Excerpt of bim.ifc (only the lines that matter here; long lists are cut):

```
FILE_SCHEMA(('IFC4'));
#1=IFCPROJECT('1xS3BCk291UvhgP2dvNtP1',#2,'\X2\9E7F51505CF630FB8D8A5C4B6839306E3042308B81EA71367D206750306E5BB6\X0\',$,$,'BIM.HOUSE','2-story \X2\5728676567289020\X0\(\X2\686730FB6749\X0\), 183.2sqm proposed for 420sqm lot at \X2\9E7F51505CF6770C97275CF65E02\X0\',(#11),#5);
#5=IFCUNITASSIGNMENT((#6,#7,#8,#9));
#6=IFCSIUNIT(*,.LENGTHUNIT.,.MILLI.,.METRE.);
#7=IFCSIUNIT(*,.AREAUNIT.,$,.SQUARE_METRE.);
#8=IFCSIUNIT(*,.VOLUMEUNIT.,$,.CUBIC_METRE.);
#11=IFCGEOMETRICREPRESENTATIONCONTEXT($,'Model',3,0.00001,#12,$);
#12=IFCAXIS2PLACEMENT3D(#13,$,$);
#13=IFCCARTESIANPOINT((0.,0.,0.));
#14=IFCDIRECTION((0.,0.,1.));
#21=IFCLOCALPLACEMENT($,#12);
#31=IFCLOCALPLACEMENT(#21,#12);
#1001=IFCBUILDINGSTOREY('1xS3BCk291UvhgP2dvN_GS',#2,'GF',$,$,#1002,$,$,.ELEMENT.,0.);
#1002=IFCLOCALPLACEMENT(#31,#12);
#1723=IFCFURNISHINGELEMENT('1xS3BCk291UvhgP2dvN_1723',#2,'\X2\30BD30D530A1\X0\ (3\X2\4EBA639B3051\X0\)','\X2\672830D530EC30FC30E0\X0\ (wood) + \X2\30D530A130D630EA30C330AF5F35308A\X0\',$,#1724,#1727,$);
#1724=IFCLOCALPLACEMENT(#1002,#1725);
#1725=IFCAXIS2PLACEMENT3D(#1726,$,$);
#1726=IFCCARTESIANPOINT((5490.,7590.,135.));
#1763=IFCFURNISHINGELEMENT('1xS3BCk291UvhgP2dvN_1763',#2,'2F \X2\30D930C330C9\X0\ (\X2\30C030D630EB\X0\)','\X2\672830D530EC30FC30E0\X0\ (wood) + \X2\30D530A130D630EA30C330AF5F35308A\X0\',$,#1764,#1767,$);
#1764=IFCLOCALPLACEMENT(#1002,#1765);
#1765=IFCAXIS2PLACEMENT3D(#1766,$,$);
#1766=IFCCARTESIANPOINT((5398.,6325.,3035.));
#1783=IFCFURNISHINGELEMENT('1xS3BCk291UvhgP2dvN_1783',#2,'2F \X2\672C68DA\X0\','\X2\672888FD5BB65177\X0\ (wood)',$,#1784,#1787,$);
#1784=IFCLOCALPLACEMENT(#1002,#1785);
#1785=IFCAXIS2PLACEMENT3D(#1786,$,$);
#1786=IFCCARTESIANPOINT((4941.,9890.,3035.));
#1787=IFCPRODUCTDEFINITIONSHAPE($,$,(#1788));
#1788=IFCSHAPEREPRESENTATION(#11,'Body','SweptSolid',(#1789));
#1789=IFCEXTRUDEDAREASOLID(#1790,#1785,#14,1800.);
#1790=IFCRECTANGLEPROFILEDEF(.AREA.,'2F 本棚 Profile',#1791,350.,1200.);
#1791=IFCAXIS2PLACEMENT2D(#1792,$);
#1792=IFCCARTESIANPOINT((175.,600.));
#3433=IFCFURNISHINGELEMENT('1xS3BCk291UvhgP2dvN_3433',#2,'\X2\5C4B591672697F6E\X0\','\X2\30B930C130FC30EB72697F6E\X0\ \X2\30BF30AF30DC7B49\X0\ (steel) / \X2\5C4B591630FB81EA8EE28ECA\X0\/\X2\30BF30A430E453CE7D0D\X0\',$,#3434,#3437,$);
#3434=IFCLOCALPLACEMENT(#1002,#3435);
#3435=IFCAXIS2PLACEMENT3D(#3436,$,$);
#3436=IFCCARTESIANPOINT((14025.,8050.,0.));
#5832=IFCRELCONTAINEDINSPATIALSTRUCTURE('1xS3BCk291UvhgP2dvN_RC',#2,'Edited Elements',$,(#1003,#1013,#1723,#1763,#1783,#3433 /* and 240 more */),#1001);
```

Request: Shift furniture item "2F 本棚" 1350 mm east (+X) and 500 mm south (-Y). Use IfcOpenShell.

```python
import ifcopenshell
import ifcopenshell.api.geometry
import ifcopenshell.util.placement
import ifcopenshell.util.unit

model = ifcopenshell.open("bim.ifc")
unit_scale = ifcopenshell.util.unit.calculate_unit_scale(model)

item = model.by_guid("1xS3BCk291UvhgP2dvN_1783")
matrix = ifcopenshell.util.placement.get_local_placement(item.ObjectPlacement)
matrix[0, 3] += 1.35 / unit_scale
matrix[1, 3] -= 0.5 / unit_scale
ifcopenshell.api.geometry.edit_object_placement(model, product=item, matrix=matrix, is_si=False)

print(ifcopenshell.util.placement.get_local_placement(item.ObjectPlacement).round(3) + 0.0)

model.write("bim_edited.ifc")
```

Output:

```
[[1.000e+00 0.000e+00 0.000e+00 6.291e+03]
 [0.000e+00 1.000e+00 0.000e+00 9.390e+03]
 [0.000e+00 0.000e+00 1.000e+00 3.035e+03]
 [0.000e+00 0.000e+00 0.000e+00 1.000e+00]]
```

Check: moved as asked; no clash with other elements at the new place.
